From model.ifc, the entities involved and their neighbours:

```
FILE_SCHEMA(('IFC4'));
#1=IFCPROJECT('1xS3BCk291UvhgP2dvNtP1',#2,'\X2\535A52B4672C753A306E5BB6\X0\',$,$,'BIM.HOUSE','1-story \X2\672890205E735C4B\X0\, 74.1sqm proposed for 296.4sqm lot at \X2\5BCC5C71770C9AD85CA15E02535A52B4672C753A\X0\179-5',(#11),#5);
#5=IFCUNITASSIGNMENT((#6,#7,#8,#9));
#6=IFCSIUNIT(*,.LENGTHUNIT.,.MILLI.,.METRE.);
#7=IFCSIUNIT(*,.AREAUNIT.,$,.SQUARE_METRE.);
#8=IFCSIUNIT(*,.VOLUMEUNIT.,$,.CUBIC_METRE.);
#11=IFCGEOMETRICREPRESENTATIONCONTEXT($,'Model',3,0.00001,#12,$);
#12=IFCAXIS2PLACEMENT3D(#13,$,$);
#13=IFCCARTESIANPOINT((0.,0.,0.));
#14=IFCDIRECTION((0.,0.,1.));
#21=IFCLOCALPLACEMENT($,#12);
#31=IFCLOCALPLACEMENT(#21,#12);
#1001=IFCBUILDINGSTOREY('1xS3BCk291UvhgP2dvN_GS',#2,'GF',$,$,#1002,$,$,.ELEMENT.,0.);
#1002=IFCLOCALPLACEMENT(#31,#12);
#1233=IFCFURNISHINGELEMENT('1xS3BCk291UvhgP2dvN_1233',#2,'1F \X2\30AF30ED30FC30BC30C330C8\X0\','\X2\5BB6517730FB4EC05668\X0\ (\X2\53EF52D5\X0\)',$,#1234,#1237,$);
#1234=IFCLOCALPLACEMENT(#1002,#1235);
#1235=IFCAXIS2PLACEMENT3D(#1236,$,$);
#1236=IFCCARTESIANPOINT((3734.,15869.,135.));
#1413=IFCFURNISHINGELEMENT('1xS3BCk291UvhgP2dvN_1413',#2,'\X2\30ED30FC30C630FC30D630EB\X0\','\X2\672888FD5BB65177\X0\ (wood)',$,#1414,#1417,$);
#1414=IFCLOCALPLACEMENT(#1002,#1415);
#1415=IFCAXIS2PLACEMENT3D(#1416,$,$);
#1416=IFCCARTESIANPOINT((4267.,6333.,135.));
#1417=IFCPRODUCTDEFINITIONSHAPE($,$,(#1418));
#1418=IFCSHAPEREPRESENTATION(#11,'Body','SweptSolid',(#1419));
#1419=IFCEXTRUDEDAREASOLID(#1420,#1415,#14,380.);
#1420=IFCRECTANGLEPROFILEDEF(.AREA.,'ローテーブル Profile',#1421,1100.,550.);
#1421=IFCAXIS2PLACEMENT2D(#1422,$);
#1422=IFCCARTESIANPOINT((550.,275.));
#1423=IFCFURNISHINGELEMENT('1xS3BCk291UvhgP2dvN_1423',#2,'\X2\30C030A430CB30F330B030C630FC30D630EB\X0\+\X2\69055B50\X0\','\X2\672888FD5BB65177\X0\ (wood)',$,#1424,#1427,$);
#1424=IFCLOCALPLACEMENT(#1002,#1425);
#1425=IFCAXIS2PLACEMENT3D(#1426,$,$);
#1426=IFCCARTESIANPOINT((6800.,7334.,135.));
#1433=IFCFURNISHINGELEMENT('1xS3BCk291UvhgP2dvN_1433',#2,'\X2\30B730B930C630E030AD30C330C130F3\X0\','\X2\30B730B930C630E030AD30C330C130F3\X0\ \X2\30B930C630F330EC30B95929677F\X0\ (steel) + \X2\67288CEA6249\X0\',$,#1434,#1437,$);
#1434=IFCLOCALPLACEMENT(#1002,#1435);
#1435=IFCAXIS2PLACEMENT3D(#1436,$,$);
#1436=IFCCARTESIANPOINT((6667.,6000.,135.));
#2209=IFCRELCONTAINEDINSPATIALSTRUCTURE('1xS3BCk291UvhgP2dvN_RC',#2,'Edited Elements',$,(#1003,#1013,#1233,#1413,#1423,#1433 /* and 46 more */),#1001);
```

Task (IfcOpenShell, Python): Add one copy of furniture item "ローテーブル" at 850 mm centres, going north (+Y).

```python
import numpy as np
import ifcopenshell
import ifcopenshell.api.geometry
import ifcopenshell.api.root
import ifcopenshell.util.element
import ifcopenshell.util.placement
import ifcopenshell.util.unit

model = ifcopenshell.open("model.ifc")
unit_scale = ifcopenshell.util.unit.calculate_unit_scale(model)


def reuse_history(source, copy):
    """copy_class also copies each property set's owner history, people and application; keep the originals."""
    for rel in copy.IsDefinedBy:
        if rel.is_a("IfcRelDefinesByProperties") and (history := rel.RelatingPropertyDefinition.OwnerHistory):
            rel.RelatingPropertyDefinition.OwnerHistory = source.OwnerHistory
            ifcopenshell.util.element.remove_deep2(model, history)


source = model.by_guid("1xS3BCk291UvhgP2dvN_1413")
base = ifcopenshell.util.placement.get_local_placement(source.ObjectPlacement)
step = np.array([0.0, 1.0, 0.0]) * 0.85 / unit_scale

for i in range(1, 2):
    copy = ifcopenshell.api.root.copy_class(model, product=source)
    copy.Representation = ifcopenshell.util.element.copy_deep(
        model, source.Representation, exclude=["IfcGeometricRepresentationContext", "IfcRepresentationMap"]
    )
    reuse_history(source, copy)
    matrix = base.copy()
    matrix[:3, 3] += i * step
    print("added at", matrix[:3, 3].round(3) + 0.0)
    ifcopenshell.api.geometry.edit_object_placement(model, product=copy, matrix=matrix, is_si=False)

model.write("model_edited.ifc")
```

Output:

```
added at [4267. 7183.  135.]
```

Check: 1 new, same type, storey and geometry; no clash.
